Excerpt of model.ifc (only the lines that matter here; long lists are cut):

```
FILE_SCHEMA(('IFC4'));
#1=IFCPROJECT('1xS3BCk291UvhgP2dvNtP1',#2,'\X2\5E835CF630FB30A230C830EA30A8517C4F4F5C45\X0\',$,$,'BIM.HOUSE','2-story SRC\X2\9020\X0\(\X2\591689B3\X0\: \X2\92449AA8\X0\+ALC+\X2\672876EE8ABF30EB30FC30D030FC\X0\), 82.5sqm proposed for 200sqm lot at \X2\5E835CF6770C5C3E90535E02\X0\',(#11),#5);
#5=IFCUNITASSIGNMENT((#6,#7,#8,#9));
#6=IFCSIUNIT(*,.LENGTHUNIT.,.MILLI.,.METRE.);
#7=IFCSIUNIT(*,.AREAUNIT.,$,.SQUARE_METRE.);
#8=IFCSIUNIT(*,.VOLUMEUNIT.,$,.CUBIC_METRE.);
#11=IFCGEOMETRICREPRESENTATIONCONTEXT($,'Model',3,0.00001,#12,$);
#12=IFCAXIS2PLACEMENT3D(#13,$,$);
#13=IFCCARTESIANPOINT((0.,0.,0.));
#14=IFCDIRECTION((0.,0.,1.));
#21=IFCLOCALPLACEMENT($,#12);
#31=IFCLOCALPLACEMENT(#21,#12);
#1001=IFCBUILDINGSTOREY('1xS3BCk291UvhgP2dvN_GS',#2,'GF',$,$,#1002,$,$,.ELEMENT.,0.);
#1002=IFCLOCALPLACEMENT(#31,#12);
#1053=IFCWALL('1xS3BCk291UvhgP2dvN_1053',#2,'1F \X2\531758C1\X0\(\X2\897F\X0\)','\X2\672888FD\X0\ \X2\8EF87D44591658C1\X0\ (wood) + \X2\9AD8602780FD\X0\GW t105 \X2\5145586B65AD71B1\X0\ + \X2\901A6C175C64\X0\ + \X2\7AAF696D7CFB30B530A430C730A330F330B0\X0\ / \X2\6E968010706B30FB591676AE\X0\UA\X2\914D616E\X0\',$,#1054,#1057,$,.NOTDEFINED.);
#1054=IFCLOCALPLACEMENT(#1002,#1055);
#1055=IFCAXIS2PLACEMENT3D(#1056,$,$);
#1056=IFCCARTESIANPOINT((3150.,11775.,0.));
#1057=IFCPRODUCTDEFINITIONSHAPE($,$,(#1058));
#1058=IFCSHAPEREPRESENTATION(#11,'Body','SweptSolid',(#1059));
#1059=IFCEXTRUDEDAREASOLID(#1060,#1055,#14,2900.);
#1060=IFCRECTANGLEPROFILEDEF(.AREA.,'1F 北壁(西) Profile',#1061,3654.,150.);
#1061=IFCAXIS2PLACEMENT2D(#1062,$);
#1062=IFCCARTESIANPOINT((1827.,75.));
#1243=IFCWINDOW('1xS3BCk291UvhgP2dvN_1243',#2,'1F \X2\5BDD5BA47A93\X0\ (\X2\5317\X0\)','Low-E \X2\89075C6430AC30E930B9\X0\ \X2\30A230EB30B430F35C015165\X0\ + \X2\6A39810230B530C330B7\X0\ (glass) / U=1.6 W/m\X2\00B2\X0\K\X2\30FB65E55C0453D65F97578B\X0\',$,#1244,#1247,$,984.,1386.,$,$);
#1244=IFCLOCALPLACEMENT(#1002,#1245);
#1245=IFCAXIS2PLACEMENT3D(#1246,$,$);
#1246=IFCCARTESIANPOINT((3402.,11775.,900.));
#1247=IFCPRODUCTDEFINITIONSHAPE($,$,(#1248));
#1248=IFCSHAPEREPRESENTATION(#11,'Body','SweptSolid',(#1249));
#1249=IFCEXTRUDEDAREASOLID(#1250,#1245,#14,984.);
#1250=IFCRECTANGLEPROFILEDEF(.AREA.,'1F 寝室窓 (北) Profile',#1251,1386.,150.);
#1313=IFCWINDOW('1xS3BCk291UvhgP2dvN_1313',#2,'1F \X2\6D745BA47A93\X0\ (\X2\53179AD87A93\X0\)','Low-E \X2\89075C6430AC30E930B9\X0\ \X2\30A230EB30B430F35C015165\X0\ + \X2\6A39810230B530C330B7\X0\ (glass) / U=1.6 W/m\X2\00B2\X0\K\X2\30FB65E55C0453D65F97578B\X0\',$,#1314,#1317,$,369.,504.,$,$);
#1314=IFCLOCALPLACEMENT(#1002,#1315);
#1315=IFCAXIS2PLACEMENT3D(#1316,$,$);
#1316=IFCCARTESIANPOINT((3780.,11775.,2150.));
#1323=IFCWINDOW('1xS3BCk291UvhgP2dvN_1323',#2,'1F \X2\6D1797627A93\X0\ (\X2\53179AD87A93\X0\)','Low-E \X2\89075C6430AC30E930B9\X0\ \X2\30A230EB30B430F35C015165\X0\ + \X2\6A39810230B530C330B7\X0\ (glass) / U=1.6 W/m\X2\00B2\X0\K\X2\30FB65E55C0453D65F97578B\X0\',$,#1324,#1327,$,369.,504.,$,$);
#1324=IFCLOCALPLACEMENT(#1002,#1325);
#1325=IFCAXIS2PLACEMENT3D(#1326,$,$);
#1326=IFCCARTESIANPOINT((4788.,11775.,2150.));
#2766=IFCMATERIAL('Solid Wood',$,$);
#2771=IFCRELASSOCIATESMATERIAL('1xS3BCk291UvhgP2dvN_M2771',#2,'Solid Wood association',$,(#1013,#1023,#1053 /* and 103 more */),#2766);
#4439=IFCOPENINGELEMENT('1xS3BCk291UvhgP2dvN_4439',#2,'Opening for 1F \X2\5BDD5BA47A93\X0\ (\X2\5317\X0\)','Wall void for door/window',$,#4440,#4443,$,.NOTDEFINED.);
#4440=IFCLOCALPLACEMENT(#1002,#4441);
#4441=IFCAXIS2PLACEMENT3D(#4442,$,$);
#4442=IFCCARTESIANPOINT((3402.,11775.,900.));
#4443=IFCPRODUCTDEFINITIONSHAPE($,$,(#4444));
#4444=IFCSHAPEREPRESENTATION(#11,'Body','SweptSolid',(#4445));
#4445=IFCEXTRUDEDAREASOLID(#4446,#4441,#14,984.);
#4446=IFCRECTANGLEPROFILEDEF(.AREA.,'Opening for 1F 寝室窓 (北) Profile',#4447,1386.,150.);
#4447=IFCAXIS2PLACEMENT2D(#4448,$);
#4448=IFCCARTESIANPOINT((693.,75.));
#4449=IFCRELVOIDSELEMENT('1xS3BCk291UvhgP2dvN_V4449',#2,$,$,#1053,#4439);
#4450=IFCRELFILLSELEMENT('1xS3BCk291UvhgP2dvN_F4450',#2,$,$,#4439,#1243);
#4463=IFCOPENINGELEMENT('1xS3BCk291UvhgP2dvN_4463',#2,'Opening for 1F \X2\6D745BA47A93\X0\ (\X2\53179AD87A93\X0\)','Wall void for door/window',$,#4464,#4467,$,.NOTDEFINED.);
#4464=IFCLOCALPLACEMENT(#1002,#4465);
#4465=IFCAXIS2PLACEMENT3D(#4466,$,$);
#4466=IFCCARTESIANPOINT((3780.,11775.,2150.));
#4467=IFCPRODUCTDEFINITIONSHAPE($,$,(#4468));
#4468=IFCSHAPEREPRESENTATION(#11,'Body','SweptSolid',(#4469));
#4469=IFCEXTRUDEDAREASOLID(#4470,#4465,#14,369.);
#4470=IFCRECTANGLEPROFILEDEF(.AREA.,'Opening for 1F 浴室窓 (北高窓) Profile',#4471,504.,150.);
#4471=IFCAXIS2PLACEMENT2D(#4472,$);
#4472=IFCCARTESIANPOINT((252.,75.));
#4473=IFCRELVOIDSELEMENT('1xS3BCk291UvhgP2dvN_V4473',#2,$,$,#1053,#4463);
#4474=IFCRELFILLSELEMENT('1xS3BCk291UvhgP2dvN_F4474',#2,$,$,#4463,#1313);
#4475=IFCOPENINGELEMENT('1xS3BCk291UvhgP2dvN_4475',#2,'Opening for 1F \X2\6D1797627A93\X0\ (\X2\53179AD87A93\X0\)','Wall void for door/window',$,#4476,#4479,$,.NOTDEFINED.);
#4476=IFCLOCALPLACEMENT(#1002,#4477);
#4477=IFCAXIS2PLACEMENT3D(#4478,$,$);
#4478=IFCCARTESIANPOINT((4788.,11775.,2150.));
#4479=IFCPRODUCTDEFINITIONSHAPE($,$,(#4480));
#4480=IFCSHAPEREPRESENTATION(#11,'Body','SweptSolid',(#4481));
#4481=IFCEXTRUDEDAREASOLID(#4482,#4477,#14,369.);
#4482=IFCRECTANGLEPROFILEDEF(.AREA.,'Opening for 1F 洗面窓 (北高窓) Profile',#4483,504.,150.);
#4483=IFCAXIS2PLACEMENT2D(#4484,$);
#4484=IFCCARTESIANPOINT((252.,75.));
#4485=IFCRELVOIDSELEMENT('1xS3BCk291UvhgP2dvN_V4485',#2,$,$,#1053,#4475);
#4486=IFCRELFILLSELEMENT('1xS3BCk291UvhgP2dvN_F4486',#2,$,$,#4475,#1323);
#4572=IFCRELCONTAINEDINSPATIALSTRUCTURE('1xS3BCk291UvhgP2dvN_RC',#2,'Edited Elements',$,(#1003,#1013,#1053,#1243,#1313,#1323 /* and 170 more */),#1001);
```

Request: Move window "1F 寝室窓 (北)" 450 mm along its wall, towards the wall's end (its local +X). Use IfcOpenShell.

```python
import ifcopenshell
import ifcopenshell.api.geometry
import ifcopenshell.util.placement
import ifcopenshell.util.unit

model = ifcopenshell.open("model.ifc")
unit_scale = ifcopenshell.util.unit.calculate_unit_scale(model)

window = model.by_guid("1xS3BCk291UvhgP2dvN_1243")
opening = window.FillsVoids[0].RelatingOpeningElement
wall = opening.VoidsElements[0].RelatingBuildingElement

wall_matrix = ifcopenshell.util.placement.get_local_placement(wall.ObjectPlacement)
shift = wall_matrix[:3, 0] * 0.45 / unit_scale
before = ifcopenshell.util.placement.get_local_placement(window.ObjectPlacement)[:3, 3].copy()

# The window is not placed relative to its opening, so move both.
for product in (opening, window):
    matrix = ifcopenshell.util.placement.get_local_placement(product.ObjectPlacement)
    matrix[:3, 3] += shift
    ifcopenshell.api.geometry.edit_object_placement(model, product=product, matrix=matrix, is_si=False)

after = ifcopenshell.util.placement.get_local_placement(window.ObjectPlacement)[:3, 3]
print("window moved by", (after - before).round(3) + 0.0)

model.write("model_rev.ifc")
```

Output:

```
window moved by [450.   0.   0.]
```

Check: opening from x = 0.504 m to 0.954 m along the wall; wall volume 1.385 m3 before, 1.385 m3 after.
